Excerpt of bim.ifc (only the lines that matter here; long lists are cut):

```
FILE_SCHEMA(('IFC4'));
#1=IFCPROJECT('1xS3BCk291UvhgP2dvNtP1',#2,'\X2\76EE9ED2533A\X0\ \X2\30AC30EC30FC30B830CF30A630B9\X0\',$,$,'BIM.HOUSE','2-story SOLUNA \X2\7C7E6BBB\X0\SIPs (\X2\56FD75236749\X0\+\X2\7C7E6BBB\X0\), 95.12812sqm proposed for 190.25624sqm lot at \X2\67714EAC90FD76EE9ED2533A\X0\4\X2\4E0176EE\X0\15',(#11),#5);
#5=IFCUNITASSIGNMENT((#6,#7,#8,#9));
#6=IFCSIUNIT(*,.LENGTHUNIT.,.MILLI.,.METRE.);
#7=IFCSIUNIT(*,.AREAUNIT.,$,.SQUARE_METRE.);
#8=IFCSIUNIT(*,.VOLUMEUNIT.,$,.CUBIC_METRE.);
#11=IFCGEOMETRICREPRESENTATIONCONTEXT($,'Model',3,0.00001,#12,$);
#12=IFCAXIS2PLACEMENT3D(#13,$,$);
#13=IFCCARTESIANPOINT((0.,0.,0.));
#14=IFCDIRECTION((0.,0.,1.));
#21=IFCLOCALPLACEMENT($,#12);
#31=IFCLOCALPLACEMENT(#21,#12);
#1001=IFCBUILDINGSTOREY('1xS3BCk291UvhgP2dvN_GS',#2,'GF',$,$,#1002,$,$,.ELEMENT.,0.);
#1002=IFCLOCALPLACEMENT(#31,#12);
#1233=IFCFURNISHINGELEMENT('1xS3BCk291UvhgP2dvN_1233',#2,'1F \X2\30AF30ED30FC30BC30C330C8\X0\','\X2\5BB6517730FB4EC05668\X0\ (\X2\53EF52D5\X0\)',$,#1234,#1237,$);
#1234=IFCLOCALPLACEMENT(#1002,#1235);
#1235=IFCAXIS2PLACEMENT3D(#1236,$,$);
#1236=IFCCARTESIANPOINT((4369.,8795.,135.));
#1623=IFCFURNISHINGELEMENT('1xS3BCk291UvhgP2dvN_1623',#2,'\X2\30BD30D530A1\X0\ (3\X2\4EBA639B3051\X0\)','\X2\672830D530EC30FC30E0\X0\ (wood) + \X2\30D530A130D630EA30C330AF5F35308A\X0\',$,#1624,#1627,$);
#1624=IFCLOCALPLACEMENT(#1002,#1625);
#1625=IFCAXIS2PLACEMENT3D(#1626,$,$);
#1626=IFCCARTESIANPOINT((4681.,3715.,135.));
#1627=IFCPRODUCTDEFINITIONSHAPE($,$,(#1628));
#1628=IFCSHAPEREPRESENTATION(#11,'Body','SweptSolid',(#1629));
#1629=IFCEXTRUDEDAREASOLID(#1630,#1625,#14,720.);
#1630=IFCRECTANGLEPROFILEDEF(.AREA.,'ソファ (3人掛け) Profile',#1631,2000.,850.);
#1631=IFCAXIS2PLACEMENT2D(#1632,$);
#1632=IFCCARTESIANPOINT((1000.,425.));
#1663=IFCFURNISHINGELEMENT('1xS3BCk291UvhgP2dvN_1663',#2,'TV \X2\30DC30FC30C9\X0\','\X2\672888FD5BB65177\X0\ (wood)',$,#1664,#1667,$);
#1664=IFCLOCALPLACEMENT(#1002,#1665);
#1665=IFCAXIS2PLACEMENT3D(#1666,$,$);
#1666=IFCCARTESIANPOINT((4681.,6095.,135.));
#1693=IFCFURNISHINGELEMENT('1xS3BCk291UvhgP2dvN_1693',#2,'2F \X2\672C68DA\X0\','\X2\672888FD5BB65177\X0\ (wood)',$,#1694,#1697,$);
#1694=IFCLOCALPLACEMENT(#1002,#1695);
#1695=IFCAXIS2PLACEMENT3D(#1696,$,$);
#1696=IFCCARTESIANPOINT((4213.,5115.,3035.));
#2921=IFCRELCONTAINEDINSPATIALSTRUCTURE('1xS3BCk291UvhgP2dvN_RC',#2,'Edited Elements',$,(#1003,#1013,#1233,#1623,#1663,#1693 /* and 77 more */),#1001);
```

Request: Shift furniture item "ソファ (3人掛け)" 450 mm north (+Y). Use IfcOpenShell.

```python
import ifcopenshell
import ifcopenshell.api.geometry
import ifcopenshell.util.placement
import ifcopenshell.util.unit

model = ifcopenshell.open("bim.ifc")
unit_scale = ifcopenshell.util.unit.calculate_unit_scale(model)

item = model.by_guid("1xS3BCk291UvhgP2dvN_1623")
matrix = ifcopenshell.util.placement.get_local_placement(item.ObjectPlacement)
matrix[1, 3] += 0.45 / unit_scale
ifcopenshell.api.geometry.edit_object_placement(model, product=item, matrix=matrix, is_si=False)

print(ifcopenshell.util.placement.get_local_placement(item.ObjectPlacement).round(3) + 0.0)

model.write("bim_v2.ifc")
```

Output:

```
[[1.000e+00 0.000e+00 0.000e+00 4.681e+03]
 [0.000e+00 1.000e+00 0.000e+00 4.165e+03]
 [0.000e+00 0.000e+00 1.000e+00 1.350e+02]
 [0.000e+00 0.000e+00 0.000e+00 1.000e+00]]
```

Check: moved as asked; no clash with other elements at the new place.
